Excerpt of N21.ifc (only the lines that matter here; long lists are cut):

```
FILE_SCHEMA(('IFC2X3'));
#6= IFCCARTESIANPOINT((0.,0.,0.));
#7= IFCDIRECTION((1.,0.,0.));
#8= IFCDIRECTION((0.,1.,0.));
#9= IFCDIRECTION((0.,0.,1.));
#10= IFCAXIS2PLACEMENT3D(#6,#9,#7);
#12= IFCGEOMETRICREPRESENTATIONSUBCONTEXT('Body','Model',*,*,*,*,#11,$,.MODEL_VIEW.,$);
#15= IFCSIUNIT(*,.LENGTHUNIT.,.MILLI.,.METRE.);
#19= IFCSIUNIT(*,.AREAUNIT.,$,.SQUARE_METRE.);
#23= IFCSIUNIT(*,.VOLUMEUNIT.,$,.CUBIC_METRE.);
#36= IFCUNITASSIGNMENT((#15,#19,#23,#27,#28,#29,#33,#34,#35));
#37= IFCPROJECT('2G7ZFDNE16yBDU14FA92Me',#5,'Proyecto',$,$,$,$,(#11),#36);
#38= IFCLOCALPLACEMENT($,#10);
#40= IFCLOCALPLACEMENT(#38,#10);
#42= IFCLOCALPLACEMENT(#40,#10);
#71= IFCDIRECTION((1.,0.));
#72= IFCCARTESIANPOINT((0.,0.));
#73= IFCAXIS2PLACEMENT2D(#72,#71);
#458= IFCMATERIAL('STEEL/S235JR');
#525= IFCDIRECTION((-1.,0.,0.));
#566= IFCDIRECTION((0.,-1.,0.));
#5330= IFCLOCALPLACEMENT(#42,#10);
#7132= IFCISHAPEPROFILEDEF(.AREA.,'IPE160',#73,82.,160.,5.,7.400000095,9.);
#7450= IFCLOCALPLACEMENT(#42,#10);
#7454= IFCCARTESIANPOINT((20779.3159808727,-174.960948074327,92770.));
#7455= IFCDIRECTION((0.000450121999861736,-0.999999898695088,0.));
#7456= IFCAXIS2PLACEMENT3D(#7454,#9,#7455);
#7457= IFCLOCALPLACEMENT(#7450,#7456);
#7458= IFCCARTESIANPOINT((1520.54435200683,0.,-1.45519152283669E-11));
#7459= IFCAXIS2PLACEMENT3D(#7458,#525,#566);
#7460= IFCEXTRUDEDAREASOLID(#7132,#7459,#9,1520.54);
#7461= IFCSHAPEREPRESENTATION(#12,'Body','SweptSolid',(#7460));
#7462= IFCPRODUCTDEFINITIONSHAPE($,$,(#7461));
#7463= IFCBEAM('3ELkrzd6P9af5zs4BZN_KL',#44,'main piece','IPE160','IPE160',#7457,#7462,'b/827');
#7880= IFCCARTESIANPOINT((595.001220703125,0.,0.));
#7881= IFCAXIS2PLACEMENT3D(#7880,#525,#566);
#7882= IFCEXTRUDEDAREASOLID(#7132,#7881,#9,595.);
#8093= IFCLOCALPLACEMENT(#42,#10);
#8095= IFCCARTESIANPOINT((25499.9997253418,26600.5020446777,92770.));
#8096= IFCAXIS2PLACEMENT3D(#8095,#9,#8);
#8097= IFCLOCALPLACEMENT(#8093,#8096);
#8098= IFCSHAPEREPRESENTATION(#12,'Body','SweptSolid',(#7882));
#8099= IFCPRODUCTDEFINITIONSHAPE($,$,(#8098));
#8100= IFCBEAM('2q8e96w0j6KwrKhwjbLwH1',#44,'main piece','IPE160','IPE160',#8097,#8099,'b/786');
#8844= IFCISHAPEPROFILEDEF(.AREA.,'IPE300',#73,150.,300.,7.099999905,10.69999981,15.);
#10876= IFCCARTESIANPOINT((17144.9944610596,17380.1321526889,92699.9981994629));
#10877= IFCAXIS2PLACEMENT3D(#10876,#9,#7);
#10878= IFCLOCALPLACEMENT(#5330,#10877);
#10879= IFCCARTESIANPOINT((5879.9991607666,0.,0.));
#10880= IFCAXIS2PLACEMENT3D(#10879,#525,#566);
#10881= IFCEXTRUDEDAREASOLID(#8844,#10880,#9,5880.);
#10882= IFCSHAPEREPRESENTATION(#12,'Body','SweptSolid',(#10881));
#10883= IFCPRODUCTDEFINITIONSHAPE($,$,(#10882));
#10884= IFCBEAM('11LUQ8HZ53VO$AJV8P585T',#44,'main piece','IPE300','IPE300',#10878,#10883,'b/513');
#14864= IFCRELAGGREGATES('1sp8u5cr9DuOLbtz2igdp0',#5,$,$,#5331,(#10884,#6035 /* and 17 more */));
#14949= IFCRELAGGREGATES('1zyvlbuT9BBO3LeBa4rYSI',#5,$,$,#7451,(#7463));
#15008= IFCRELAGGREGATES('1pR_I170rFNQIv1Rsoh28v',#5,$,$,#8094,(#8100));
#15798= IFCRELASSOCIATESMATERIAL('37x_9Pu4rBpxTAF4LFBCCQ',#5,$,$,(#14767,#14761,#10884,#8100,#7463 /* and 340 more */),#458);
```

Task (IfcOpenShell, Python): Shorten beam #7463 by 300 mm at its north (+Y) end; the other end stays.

```python
import ifcopenshell
import ifcopenshell.util.representation

model = ifcopenshell.open("N21.ifc")

member = model.by_id(7463)
change = -300.0

# The extrusion runs towards the end named, so only its depth changes.
body = ifcopenshell.util.representation.get_representation(member, "Model", "Body")
solid = body.Items[0]
old_length = solid.Depth
solid.Depth += change

print(f"length {old_length:g} -> {solid.Depth:g}")

model.write("N21_edited.ifc")
```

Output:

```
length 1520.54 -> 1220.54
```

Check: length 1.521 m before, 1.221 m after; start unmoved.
